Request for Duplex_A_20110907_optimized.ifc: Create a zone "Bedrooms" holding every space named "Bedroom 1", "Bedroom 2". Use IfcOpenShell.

First a look at what the model holds.

```python
import ifcopenshell

model = ifcopenshell.open("Duplex_A_20110907_optimized.ifc")
print(model.schema)
seen = {}
for space in model.by_type("IfcSpace"):
    seen[space.LongName] = seen.get(space.LongName, 0) + 1
for name, count in sorted(seen.items(), key=str):
    print(count, "x", name)
print("zones:", [z.Name for z in model.by_type("IfcZone")][:20])
```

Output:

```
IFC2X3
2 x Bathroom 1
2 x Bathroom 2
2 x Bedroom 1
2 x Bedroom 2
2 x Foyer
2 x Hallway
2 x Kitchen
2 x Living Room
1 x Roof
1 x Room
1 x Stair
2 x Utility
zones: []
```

```python
import ifcopenshell
import ifcopenshell.api.group
import ifcopenshell.api.root

model = ifcopenshell.open("Duplex_A_20110907_optimized.ifc")

names = {"Bedroom 1", "Bedroom 2"}
spaces = [s for s in model.by_type("IfcSpace") if s.LongName in names]

zone = ifcopenshell.api.root.create_entity(model, ifc_class="IfcZone", name="Bedrooms")
ifcopenshell.api.group.assign_group(model, products=spaces, group=zone)
print(len(spaces), "spaces in", zone.Name)

model.write("Duplex_A_20110907_optimized_edited.ifc")
```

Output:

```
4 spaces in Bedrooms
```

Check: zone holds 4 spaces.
